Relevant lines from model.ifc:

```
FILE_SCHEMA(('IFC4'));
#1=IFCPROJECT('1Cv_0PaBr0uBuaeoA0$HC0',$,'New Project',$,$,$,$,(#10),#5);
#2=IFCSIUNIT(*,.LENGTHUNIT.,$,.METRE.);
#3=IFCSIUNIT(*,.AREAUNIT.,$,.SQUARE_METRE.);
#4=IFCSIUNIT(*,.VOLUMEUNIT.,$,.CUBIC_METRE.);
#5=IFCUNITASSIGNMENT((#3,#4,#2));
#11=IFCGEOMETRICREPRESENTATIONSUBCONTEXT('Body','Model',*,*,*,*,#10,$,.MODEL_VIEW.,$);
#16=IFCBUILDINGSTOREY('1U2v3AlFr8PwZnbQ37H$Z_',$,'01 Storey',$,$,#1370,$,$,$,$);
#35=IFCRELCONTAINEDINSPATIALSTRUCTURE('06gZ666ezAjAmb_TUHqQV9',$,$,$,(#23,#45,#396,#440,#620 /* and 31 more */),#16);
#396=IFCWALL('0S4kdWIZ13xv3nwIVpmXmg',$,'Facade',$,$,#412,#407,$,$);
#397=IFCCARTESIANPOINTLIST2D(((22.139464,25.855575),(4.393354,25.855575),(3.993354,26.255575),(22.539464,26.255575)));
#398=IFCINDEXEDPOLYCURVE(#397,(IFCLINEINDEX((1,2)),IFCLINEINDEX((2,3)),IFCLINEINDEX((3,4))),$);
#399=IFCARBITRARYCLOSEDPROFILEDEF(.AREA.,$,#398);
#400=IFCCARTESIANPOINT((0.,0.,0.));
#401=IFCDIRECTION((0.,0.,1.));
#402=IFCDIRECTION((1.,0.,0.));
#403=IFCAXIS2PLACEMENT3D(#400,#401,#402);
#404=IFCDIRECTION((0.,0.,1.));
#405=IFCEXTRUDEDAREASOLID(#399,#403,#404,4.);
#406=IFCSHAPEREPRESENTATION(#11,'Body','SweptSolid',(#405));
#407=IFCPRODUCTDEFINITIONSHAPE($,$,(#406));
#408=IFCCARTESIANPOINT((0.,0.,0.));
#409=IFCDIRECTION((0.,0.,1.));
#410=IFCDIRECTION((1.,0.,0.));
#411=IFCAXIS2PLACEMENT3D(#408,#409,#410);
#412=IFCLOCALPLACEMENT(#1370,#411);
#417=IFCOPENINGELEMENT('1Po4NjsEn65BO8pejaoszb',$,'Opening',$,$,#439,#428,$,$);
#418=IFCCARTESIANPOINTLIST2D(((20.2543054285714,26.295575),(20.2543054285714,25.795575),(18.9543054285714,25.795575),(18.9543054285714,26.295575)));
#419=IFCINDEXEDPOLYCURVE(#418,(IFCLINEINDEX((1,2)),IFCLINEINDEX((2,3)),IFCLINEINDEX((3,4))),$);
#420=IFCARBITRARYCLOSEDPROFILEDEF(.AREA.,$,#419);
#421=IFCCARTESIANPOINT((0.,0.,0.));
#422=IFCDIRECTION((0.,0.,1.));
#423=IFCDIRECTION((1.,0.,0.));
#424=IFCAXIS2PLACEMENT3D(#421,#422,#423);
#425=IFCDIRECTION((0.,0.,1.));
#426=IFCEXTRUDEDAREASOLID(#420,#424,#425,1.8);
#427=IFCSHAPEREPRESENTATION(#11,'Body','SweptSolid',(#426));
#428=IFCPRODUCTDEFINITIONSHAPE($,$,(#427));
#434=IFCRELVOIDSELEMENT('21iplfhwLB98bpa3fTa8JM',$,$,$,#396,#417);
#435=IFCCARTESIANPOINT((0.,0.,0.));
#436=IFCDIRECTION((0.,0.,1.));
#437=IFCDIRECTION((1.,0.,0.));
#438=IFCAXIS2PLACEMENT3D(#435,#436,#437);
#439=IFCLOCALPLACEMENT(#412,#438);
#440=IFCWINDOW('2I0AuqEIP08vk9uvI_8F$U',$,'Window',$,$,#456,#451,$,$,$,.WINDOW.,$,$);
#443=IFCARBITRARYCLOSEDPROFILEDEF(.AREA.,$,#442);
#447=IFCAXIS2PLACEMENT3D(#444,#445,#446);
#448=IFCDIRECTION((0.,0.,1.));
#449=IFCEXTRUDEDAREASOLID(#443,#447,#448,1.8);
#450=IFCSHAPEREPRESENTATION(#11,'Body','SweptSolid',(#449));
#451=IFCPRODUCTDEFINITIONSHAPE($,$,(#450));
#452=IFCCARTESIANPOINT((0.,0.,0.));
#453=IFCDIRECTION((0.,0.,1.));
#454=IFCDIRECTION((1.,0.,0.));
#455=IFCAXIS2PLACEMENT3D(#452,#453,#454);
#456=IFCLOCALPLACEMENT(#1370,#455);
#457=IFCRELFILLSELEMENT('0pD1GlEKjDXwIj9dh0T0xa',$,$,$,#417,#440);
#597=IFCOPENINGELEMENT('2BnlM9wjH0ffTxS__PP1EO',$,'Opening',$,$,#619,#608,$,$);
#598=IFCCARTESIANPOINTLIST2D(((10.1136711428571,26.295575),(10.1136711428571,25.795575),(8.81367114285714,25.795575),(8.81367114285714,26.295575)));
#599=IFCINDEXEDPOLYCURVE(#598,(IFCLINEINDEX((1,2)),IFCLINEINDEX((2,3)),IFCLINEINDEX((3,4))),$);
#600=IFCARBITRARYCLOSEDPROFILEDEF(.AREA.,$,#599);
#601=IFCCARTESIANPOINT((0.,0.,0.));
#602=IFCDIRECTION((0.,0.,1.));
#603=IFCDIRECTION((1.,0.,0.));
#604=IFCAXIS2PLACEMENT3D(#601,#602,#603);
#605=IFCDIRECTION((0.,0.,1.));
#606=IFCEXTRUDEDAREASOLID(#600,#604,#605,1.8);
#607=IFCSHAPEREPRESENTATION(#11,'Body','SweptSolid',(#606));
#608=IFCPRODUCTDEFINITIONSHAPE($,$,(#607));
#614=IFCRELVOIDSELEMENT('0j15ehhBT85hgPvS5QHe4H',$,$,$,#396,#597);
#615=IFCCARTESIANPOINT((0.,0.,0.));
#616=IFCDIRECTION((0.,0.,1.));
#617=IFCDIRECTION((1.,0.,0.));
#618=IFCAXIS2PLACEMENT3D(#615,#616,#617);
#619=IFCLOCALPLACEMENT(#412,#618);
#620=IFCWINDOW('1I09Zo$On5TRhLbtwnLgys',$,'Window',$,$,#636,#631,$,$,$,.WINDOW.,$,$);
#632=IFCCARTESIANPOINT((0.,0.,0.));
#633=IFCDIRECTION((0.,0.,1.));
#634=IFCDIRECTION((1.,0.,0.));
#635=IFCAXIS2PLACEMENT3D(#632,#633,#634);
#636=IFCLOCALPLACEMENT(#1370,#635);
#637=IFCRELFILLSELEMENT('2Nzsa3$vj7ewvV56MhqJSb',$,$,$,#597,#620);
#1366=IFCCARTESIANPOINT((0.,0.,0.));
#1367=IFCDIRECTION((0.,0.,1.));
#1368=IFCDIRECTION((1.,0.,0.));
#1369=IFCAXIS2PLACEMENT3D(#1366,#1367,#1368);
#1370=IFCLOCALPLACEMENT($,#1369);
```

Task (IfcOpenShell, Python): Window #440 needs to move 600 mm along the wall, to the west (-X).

```python
import ifcopenshell
import ifcopenshell.api.geometry
import ifcopenshell.util.placement
import ifcopenshell.util.unit

model = ifcopenshell.open("model.ifc")
unit_scale = ifcopenshell.util.unit.calculate_unit_scale(model)

window = model.by_guid("2I0AuqEIP08vk9uvI_8F$U")
opening = window.FillsVoids[0].RelatingOpeningElement
wall = opening.VoidsElements[0].RelatingBuildingElement

wall_matrix = ifcopenshell.util.placement.get_local_placement(wall.ObjectPlacement)
shift = wall_matrix[:3, 0] * -0.6 / unit_scale
before = ifcopenshell.util.placement.get_local_placement(window.ObjectPlacement)[:3, 3].copy()

# The window is not placed relative to its opening, so move both.
for product in (opening, window):
    matrix = ifcopenshell.util.placement.get_local_placement(product.ObjectPlacement)
    matrix[:3, 3] += shift
    ifcopenshell.api.geometry.edit_object_placement(model, product=product, matrix=matrix, is_si=False)

after = ifcopenshell.util.placement.get_local_placement(window.ObjectPlacement)[:3, 3]
print("window moved by", (after - before).round(3) + 0.0)

model.write("model-out.ifc")
```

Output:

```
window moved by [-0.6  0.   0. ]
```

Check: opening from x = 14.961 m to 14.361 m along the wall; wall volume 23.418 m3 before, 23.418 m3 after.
